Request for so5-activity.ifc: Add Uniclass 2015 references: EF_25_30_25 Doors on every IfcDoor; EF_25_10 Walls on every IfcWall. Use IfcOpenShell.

First a look at what the model holds.

```python
import ifcopenshell

model = ifcopenshell.open("so5-activity.ifc")
print(model.schema)
print("classifications:", [c.Name for c in model.by_type("IfcClassification")])
for ifc_class in ("IfcDoor", "IfcRoof", "IfcStair", "IfcWall", "IfcWindow"):
    print(ifc_class, len(model.by_type(ifc_class)))
```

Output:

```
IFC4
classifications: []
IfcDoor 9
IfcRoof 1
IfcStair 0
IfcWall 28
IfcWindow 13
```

```python
import ifcopenshell
import ifcopenshell.api.classification

model = ifcopenshell.open("so5-activity.ifc")

system = ifcopenshell.api.classification.add_classification(model, classification="Uniclass 2015")

codes = {
    "IfcDoor": ("EF_25_30_25", "Doors"),
    "IfcWall": ("EF_25_10", "Walls"),
}
for ifc_class, (code, name) in codes.items():
    products = model.by_type(ifc_class)
    ifcopenshell.api.classification.add_reference(
        model, products=products, classification=system, identification=code, name=name
    )
    print(code, len(products))

model.write("so5-activity_updated.ifc")
```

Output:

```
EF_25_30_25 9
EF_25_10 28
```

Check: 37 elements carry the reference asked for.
